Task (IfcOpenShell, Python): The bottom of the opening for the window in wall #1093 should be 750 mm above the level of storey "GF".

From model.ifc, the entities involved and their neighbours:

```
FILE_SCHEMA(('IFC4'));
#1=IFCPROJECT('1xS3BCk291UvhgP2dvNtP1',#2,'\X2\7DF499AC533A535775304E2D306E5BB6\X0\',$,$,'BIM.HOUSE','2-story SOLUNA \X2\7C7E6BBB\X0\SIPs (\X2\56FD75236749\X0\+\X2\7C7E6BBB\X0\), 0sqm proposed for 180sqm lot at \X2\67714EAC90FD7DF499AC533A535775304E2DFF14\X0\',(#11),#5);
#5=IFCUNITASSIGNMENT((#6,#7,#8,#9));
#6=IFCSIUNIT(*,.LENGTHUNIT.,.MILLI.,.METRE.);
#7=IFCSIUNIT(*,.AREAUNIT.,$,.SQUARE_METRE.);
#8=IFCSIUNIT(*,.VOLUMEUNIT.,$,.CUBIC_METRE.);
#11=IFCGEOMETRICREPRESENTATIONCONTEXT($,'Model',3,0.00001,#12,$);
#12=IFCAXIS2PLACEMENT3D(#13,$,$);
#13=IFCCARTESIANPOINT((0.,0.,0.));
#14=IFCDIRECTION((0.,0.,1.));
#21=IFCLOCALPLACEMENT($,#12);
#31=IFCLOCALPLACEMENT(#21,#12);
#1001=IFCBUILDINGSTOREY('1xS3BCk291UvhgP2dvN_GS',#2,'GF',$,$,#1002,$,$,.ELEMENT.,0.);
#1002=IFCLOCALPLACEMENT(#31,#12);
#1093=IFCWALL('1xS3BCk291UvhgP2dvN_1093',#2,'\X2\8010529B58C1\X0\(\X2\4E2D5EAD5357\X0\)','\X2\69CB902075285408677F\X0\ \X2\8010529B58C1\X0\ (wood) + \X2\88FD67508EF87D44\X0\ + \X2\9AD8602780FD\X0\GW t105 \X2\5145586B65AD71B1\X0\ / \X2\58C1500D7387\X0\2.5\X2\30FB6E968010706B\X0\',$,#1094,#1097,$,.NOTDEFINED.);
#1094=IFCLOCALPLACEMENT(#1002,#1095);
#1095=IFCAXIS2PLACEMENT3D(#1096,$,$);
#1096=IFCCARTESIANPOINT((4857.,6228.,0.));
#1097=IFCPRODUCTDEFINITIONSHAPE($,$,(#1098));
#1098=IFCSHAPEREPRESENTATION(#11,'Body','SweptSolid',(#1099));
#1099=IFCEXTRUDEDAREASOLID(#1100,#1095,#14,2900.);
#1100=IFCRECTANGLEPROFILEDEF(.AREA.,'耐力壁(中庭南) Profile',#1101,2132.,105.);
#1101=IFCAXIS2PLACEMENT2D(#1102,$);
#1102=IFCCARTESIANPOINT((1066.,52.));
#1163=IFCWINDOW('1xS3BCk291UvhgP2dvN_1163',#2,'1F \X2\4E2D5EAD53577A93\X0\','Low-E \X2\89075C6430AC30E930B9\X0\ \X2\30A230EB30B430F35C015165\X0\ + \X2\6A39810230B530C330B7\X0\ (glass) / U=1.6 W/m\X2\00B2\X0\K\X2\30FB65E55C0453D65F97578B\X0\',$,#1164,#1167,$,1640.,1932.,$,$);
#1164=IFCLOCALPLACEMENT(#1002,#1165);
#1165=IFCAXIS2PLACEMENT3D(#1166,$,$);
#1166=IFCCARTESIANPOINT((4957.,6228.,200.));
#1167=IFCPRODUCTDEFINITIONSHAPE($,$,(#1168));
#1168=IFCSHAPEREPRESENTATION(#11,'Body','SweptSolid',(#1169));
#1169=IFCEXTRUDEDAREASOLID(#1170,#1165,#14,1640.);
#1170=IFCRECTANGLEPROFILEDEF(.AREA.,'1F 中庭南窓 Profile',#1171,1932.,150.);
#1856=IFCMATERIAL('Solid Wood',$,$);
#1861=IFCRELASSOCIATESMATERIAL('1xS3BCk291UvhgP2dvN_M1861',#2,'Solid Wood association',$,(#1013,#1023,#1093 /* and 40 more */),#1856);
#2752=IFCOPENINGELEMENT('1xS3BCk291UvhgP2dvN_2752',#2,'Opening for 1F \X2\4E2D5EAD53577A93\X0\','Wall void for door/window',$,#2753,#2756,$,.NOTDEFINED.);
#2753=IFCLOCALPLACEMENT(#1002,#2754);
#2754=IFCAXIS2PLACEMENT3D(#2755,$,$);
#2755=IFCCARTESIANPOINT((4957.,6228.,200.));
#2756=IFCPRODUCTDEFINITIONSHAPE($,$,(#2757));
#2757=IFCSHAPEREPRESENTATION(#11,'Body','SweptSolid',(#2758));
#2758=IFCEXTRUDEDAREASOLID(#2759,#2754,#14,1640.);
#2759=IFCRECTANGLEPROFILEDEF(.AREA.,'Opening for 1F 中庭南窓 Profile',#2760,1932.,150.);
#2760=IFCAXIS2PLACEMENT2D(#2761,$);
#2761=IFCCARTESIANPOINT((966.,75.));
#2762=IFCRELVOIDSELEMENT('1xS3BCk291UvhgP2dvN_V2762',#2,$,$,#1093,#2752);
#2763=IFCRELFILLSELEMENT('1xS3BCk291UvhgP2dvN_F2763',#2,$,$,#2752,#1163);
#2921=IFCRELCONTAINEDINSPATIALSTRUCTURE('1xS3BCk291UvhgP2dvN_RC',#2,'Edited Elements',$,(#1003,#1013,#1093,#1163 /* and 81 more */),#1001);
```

```python
import numpy as np
import ifcopenshell
import ifcopenshell.api.geometry
import ifcopenshell.geom
import ifcopenshell.util.element
import ifcopenshell.util.placement
import ifcopenshell.util.shape
import ifcopenshell.util.unit

model = ifcopenshell.open("model.ifc")
unit_scale = ifcopenshell.util.unit.calculate_unit_scale(model)

window = model.by_guid("1xS3BCk291UvhgP2dvN_1163")
opening = window.FillsVoids[0].RelatingOpeningElement
storey = ifcopenshell.util.element.get_container(window, ifc_class="IfcBuildingStorey")
level = ifcopenshell.util.placement.get_local_placement(storey.ObjectPlacement)[2, 3]

# The opening's origin need not be at the sill, so measure its lowest point.
shape = ifcopenshell.geom.create_shape(ifcopenshell.geom.settings(), opening)
bottom = ifcopenshell.util.shape.get_shape_bottom_elevation(shape, shape.geometry) / unit_scale
dz = level + 750.0 - bottom

shift = np.array([0.0, 0.0, dz])
# The window is not placed relative to its opening, so move both.
for product in (opening, window):
    matrix = ifcopenshell.util.placement.get_local_placement(product.ObjectPlacement)
    matrix[:3, 3] += shift
    ifcopenshell.api.geometry.edit_object_placement(model, product=product, matrix=matrix, is_si=False)

print(f"moved by {dz * unit_scale:+.3f} m")

model.write("model_updated.ifc")
```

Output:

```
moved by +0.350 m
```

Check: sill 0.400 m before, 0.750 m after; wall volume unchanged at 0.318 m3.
